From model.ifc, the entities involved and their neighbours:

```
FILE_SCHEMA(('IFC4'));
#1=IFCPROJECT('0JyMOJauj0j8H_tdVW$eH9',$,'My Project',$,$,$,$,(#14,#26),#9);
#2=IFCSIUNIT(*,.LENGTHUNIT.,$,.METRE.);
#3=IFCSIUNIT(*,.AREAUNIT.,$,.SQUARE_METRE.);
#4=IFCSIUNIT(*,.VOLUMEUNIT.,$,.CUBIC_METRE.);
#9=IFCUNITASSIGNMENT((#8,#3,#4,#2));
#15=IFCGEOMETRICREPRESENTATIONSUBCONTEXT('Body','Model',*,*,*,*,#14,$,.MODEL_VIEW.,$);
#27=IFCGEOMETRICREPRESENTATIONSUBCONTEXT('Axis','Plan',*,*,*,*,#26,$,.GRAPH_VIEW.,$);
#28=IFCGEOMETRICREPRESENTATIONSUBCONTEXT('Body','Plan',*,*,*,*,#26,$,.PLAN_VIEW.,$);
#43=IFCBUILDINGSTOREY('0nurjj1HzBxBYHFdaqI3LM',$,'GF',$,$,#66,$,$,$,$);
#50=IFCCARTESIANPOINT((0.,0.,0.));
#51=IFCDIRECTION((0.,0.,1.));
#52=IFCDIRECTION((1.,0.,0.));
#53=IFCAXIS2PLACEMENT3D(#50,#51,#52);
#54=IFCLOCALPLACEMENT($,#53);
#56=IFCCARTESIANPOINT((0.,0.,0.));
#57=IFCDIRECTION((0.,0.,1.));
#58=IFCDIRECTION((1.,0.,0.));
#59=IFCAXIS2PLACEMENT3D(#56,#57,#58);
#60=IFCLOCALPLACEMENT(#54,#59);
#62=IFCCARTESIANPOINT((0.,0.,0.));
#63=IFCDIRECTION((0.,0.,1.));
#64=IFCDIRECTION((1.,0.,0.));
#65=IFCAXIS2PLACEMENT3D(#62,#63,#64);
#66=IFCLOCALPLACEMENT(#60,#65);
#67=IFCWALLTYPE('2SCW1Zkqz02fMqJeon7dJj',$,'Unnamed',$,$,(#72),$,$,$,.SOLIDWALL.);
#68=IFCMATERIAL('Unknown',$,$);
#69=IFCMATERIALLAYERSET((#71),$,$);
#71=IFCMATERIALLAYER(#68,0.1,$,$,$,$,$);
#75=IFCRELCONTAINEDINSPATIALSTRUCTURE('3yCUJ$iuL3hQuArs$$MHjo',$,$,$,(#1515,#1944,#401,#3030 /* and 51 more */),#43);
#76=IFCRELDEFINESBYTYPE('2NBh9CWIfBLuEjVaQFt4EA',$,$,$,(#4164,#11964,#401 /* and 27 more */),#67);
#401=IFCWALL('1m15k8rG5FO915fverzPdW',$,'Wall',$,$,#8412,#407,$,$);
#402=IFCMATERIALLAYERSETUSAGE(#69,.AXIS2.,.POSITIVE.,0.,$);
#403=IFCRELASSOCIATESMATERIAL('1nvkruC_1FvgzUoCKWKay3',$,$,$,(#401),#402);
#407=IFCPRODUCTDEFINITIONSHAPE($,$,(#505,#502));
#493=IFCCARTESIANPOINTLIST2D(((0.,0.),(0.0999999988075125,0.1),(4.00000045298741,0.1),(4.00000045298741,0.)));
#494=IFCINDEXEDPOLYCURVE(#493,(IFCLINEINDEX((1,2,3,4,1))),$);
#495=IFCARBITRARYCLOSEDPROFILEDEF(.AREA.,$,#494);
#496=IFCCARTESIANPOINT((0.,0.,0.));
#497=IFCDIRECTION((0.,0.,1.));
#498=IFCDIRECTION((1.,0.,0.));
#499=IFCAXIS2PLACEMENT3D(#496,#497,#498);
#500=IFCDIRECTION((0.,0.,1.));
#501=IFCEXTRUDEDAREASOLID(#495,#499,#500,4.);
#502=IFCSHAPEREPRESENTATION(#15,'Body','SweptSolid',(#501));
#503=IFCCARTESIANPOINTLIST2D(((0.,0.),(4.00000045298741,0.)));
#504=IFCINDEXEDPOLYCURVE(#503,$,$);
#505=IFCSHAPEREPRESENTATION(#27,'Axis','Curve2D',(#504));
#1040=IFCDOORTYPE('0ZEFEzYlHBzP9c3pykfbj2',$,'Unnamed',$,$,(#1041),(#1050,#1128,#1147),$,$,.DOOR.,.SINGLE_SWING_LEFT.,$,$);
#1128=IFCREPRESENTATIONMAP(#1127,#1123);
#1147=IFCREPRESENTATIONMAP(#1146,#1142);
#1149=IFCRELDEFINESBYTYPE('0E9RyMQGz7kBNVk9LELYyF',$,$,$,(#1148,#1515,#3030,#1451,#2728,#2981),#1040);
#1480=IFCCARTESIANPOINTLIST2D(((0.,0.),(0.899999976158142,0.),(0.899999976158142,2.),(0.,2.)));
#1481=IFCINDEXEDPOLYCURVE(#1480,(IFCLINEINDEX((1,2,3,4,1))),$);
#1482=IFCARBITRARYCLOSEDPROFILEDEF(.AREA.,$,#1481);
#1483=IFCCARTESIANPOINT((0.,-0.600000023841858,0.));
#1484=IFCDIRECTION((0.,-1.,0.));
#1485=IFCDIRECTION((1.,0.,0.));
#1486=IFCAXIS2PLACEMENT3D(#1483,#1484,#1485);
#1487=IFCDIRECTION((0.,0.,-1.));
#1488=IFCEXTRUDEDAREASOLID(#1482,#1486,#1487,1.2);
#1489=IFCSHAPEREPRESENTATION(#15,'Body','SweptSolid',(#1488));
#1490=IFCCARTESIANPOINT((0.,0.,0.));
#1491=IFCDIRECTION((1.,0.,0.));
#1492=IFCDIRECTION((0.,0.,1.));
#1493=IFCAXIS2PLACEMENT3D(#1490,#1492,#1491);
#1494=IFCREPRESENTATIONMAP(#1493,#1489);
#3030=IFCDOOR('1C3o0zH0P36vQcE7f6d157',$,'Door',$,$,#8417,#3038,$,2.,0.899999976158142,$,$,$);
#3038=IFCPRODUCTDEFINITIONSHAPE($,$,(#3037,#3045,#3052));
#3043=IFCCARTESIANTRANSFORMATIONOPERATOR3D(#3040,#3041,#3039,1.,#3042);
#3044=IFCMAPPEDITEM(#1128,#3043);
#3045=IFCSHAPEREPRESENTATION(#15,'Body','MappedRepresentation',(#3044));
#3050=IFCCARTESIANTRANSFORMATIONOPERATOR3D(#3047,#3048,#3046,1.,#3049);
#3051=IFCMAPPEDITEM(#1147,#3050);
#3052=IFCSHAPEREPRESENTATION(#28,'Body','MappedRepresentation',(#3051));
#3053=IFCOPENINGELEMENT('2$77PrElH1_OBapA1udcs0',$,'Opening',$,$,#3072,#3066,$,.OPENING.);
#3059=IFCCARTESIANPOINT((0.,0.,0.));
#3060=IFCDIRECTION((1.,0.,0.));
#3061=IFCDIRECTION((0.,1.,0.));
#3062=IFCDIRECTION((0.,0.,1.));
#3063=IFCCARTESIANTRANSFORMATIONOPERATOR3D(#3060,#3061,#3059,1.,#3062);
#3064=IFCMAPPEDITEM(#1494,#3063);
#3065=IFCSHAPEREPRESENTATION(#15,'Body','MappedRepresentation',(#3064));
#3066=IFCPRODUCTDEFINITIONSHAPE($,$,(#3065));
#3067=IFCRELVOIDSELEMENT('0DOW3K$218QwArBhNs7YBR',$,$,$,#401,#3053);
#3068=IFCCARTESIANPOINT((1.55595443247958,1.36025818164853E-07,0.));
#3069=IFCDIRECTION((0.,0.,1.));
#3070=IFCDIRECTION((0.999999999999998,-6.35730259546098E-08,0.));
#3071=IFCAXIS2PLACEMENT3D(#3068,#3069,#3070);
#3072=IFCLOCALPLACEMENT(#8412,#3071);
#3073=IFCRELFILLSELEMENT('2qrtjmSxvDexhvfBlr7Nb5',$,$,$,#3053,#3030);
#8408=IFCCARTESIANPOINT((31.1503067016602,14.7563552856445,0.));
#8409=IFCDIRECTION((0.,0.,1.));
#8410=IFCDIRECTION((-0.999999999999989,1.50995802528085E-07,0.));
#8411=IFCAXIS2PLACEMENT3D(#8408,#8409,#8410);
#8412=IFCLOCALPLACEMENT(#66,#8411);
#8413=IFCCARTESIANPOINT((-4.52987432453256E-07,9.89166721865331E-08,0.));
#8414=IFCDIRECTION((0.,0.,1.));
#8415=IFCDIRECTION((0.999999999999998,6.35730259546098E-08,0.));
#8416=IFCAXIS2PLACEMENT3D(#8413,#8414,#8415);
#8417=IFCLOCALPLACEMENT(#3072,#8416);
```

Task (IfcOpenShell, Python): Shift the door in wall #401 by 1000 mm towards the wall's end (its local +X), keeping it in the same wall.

```python
import ifcopenshell
import ifcopenshell.api.geometry
import ifcopenshell.util.placement
import ifcopenshell.util.unit

model = ifcopenshell.open("model.ifc")
unit_scale = ifcopenshell.util.unit.calculate_unit_scale(model)

door = model.by_id(3030)
opening = door.FillsVoids[0].RelatingOpeningElement
wall = opening.VoidsElements[0].RelatingBuildingElement

wall_matrix = ifcopenshell.util.placement.get_local_placement(wall.ObjectPlacement)
shift = wall_matrix[:3, 0] * 1 / unit_scale
before = ifcopenshell.util.placement.get_local_placement(door.ObjectPlacement)[:3, 3].copy()

# The door is placed relative to its opening, so it follows when the opening moves.
matrix = ifcopenshell.util.placement.get_local_placement(opening.ObjectPlacement)
matrix[:3, 3] += shift
ifcopenshell.api.geometry.edit_object_placement(
    model, product=opening, matrix=matrix, is_si=False, should_transform_children=True
)

after = ifcopenshell.util.placement.get_local_placement(door.ObjectPlacement)[:3, 3]
print("door moved by", (after - before).round(3) + 0.0)

model.write("model_updated.ifc")
```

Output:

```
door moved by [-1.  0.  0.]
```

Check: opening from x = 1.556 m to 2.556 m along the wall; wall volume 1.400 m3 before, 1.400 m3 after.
